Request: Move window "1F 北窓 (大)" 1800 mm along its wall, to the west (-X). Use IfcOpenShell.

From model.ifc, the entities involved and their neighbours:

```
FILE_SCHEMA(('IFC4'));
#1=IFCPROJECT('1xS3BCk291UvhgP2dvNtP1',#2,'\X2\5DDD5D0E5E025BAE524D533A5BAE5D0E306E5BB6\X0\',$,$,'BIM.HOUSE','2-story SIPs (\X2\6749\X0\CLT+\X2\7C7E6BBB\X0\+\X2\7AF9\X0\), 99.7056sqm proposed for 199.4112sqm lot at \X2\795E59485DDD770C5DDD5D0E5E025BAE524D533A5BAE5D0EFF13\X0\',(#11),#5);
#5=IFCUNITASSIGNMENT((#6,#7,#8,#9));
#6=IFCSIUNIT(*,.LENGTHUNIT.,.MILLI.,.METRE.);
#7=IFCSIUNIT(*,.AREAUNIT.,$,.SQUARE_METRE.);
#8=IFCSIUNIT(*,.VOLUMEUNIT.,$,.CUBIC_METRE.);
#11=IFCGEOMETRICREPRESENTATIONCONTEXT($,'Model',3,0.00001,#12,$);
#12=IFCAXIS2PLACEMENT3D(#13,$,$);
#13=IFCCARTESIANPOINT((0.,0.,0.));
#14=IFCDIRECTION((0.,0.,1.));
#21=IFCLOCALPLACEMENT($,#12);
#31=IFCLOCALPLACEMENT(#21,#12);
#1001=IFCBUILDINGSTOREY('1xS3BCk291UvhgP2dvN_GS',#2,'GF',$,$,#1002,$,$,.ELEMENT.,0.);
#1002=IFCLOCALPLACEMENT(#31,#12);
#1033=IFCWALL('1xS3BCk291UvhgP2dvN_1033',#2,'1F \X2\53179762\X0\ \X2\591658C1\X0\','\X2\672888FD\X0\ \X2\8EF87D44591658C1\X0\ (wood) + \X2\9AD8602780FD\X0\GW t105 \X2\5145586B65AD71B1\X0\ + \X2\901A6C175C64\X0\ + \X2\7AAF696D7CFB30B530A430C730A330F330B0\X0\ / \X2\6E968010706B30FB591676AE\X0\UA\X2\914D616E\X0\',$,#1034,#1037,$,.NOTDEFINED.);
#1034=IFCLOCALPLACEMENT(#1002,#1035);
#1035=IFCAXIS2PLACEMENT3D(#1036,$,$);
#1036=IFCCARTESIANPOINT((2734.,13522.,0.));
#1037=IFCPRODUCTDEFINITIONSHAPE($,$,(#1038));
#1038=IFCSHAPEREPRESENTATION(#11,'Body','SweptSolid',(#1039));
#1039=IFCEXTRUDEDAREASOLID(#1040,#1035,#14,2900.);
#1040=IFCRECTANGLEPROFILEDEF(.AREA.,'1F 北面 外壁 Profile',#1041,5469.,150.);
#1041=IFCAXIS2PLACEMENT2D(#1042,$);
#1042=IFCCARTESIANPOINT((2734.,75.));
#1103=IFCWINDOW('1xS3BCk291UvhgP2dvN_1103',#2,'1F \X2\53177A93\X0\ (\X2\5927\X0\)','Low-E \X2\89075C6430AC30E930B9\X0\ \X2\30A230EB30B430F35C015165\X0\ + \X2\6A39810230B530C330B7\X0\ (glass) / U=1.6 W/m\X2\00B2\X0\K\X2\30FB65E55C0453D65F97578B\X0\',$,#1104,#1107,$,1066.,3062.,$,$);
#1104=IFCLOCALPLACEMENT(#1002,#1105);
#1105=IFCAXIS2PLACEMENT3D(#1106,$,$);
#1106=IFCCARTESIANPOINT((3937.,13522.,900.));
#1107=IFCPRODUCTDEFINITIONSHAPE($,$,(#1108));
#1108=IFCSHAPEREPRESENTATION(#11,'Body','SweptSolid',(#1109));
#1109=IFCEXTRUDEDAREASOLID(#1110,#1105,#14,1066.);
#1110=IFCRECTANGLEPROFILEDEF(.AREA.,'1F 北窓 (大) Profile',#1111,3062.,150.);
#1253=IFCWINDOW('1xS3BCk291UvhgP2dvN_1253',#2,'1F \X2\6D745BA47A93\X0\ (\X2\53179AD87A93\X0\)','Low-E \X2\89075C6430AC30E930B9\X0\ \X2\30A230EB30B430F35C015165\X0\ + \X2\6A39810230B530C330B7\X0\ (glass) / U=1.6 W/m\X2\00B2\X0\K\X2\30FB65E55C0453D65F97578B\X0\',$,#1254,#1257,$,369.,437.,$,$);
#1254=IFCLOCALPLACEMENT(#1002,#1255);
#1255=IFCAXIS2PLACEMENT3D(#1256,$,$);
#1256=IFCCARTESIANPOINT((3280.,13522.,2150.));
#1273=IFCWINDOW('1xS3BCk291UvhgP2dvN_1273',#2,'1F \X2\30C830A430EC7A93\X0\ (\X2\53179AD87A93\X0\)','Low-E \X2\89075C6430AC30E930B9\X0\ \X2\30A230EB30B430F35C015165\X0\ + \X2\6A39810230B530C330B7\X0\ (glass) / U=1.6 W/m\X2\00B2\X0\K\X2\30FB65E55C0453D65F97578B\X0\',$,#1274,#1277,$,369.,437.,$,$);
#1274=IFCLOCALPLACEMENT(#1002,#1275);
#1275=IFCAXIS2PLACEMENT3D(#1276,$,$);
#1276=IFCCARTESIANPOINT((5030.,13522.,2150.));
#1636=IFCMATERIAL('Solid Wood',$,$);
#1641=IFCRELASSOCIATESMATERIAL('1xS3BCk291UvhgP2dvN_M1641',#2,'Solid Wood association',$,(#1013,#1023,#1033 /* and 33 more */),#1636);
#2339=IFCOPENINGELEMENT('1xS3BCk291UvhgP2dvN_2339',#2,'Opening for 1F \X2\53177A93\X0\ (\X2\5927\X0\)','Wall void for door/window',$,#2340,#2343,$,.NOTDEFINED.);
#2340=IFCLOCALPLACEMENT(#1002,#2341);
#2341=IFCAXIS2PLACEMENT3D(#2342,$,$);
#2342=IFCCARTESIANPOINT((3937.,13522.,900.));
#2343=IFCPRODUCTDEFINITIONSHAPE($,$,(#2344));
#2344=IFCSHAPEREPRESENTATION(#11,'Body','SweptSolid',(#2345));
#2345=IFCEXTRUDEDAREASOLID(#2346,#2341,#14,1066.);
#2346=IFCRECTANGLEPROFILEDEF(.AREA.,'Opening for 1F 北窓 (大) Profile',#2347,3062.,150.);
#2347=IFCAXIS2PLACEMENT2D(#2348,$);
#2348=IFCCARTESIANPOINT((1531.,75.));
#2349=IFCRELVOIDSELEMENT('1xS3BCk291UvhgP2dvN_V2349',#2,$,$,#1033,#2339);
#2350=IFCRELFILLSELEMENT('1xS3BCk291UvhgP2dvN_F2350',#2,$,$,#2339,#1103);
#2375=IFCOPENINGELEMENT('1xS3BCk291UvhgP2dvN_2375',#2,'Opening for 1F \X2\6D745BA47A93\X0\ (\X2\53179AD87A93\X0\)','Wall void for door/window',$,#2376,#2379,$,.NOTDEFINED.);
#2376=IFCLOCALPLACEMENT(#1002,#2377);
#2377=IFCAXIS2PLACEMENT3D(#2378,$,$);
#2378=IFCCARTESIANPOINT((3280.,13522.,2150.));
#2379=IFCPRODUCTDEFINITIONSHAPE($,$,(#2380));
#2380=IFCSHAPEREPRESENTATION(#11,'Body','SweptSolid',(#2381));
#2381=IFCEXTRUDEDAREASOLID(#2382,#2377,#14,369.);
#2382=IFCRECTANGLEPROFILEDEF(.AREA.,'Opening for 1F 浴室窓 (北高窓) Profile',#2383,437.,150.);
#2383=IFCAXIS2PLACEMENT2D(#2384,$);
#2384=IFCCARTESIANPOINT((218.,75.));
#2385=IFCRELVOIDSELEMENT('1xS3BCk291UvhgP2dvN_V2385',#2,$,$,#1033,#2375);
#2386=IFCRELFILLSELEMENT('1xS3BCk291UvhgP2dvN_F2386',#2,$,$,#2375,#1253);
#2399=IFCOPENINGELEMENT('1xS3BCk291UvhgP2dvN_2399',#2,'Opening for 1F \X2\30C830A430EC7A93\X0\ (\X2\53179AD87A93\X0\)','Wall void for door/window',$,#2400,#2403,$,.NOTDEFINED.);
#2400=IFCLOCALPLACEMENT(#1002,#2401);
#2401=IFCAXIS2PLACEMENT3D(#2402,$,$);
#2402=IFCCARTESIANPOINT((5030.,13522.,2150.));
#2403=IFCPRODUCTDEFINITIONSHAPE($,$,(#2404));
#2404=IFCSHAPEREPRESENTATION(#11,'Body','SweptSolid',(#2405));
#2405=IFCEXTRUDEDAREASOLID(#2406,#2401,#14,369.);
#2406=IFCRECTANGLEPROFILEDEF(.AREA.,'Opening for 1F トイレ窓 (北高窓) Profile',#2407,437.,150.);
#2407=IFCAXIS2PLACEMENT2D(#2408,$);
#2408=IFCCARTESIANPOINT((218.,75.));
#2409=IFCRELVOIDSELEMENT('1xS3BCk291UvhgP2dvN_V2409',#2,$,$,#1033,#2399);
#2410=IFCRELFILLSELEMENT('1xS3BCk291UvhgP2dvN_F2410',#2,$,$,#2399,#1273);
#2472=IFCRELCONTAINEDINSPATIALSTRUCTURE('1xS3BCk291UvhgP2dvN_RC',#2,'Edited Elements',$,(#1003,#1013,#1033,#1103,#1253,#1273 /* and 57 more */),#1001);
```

```python
import ifcopenshell
import ifcopenshell.api.geometry
import ifcopenshell.util.placement

model = ifcopenshell.open("model.ifc")

window = model.by_guid("1xS3BCk291UvhgP2dvN_1103")
opening = window.FillsVoids[0].RelatingOpeningElement
wall = opening.VoidsElements[0].RelatingBuildingElement

wall_matrix = ifcopenshell.util.placement.get_local_placement(wall.ObjectPlacement)
shift = wall_matrix[:3, 0] * -1800.0
before = ifcopenshell.util.placement.get_local_placement(window.ObjectPlacement)[:3, 3].copy()

# The window is not placed relative to its opening, so move both.
for product in (opening, window):
    matrix = ifcopenshell.util.placement.get_local_placement(product.ObjectPlacement)
    matrix[:3, 3] += shift
    ifcopenshell.api.geometry.edit_object_placement(model, product=product, matrix=matrix, is_si=False)

after = ifcopenshell.util.placement.get_local_placement(window.ObjectPlacement)[:3, 3]
print("window moved by", (after - before).round(3) + 0.0)

model.write("model_edited.ifc")
```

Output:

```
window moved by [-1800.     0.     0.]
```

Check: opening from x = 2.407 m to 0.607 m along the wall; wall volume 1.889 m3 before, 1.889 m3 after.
